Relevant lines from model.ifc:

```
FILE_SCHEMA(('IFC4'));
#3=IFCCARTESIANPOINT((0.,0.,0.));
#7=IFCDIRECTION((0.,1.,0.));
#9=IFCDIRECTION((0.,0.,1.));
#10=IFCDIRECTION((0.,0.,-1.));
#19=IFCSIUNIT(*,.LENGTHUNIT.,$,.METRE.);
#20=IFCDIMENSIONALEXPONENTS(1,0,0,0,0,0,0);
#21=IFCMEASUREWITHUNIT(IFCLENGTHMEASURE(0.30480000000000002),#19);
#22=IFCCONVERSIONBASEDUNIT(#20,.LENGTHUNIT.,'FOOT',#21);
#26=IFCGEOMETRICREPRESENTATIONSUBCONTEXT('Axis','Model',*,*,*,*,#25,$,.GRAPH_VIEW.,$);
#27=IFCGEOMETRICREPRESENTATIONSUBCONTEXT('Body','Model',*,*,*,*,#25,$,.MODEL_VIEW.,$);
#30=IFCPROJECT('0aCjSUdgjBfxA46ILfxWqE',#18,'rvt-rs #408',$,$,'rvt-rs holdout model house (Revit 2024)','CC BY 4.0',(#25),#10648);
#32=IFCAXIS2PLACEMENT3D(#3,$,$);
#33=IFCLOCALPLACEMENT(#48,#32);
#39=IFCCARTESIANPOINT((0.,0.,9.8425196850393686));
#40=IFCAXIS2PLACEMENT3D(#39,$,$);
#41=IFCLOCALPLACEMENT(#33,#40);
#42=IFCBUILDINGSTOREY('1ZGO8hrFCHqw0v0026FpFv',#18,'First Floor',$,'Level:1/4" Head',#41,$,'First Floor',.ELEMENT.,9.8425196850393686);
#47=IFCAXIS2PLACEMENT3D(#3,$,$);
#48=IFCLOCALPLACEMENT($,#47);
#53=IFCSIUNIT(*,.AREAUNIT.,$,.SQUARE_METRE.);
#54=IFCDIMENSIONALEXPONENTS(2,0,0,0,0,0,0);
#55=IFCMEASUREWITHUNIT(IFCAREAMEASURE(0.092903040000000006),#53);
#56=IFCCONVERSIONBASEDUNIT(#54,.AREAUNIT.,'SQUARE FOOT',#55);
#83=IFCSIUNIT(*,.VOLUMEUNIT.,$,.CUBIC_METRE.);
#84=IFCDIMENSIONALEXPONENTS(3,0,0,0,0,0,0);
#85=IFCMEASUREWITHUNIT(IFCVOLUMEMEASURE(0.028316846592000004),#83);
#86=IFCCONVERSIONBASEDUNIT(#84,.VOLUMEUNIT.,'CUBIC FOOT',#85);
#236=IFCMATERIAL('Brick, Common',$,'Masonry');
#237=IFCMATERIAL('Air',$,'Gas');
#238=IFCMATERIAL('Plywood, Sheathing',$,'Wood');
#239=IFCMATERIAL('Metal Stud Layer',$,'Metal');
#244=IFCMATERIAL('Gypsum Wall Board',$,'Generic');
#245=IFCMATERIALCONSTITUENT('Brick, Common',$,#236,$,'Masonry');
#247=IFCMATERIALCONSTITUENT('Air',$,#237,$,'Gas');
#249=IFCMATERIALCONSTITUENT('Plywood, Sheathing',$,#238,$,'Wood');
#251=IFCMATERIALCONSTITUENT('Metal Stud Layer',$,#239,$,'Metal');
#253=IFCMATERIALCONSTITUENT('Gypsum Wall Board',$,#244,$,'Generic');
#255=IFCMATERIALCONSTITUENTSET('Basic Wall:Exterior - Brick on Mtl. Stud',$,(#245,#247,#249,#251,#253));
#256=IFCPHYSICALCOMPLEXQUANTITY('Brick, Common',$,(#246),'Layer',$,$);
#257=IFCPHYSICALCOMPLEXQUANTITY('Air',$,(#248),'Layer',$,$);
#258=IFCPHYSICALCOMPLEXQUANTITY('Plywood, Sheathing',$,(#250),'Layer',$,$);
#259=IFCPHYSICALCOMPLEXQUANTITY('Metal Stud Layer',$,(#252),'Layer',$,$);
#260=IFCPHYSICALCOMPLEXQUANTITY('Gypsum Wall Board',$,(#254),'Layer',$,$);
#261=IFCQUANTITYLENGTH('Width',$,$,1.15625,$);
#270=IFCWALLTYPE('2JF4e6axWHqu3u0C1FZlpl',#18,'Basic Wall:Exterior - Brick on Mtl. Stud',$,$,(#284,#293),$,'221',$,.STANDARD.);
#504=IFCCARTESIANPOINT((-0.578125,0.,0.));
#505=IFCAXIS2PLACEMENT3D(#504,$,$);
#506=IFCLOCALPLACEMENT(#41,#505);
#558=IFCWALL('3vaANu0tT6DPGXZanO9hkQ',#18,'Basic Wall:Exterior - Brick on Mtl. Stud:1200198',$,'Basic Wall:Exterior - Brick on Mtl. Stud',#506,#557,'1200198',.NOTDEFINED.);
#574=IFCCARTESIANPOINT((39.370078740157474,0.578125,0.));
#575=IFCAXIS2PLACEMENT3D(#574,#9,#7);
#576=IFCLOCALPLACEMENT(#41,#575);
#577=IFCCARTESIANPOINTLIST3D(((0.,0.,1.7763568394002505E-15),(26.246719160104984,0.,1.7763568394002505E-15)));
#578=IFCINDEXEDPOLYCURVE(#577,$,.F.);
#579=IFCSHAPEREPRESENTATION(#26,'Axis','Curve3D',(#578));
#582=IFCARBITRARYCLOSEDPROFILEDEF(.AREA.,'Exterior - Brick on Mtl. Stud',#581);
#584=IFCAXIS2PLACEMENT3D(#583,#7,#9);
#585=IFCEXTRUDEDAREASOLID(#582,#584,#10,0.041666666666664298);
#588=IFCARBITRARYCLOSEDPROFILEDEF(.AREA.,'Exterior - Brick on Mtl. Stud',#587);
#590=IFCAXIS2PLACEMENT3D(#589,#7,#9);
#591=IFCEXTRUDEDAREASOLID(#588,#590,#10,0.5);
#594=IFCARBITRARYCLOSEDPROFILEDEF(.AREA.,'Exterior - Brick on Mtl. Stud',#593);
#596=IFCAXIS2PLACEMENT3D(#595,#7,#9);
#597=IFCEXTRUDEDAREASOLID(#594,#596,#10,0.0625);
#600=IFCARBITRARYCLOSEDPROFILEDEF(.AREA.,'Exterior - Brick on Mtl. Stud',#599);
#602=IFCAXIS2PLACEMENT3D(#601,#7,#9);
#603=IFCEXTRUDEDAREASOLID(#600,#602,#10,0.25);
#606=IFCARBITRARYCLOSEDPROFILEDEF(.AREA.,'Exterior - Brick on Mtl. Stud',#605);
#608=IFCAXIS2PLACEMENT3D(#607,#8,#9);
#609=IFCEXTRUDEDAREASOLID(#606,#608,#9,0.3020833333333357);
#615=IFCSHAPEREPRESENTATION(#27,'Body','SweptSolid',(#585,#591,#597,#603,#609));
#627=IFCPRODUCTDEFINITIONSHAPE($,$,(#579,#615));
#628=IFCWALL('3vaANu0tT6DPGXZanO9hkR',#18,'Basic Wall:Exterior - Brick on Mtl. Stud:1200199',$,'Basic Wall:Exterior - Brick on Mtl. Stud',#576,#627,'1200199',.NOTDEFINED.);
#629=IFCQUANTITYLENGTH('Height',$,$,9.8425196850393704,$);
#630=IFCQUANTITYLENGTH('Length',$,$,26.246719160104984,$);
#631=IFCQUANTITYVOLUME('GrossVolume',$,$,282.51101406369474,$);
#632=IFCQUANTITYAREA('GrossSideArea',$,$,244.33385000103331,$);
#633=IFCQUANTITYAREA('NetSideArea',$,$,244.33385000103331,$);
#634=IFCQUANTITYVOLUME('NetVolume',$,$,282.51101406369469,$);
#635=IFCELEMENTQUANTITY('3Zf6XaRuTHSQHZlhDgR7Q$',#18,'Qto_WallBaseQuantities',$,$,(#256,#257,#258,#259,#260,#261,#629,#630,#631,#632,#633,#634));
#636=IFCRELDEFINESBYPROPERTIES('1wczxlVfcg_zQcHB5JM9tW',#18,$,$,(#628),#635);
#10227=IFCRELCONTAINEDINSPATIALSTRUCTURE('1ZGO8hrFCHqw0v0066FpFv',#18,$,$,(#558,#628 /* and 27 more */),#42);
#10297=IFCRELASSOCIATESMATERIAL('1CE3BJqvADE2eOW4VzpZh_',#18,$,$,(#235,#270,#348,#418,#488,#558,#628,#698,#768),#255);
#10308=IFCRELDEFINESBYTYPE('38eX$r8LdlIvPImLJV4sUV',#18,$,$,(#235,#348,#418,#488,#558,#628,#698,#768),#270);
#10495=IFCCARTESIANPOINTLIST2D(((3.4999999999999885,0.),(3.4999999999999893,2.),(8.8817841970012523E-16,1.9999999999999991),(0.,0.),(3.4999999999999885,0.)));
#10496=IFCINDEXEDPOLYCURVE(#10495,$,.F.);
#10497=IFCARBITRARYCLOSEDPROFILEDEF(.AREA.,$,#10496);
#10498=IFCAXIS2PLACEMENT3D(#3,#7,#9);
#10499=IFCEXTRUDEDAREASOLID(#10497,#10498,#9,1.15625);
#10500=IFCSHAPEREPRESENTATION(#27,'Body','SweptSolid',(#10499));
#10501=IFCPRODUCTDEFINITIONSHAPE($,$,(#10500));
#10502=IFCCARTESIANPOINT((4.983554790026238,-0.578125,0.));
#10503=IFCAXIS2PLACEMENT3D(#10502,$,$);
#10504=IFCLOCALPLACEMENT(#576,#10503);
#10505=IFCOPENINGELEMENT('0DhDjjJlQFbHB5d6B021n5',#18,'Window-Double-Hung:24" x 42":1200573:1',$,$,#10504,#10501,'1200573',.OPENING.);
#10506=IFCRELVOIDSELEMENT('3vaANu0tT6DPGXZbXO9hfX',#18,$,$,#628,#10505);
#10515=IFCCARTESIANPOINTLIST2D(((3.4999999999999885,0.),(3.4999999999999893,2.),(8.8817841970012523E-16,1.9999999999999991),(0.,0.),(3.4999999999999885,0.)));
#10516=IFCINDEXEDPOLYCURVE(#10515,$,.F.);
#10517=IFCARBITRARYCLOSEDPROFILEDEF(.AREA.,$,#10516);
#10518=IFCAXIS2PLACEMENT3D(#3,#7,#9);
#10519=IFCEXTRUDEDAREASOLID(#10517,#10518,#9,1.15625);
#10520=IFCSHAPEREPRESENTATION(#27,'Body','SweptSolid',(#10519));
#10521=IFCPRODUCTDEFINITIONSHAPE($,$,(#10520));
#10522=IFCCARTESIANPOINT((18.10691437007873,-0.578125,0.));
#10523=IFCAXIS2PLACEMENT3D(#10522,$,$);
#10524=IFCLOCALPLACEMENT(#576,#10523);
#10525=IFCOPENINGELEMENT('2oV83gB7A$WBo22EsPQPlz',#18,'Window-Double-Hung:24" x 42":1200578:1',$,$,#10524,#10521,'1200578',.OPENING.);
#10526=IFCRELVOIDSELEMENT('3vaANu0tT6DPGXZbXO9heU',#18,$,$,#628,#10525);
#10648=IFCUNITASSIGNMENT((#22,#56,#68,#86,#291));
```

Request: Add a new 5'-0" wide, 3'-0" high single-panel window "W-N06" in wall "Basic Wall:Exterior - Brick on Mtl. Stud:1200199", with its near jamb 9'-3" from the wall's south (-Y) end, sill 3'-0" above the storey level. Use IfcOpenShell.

```python
import numpy as np
import ifcopenshell
import ifcopenshell.api.feature
import ifcopenshell.api.geometry
import ifcopenshell.api.pset
import ifcopenshell.api.root
import ifcopenshell.api.spatial
import ifcopenshell.geom
import ifcopenshell.util.element
import ifcopenshell.util.placement
import ifcopenshell.util.representation
import ifcopenshell.util.shape
import ifcopenshell.util.unit

model = ifcopenshell.open("model.ifc")
unit_scale = ifcopenshell.util.unit.calculate_unit_scale(model)
area_scale = ifcopenshell.util.unit.calculate_unit_scale(model, "AREAUNIT")
volume_scale = ifcopenshell.util.unit.calculate_unit_scale(model, "VOLUMEUNIT")
settings = ifcopenshell.geom.settings()


def volume(element):
    """Net volume in cubic metres, openings subtracted."""
    shape = ifcopenshell.geom.create_shape(settings, element)
    return ifcopenshell.util.shape.get_volume(shape.geometry)


wall = model.by_guid("3vaANu0tT6DPGXZanO9hkR")
storey = ifcopenshell.util.element.get_container(wall, ifc_class="IfcBuildingStorey")
context = ifcopenshell.util.representation.get_context(model, "Model", "Body", "MODEL_VIEW")
before = volume(wall)

width, height, from_end, sill = 1.524, 0.9144, 2.8194, 0.9144  # metres

# The wall runs along its own X axis, and the end named is its -X end.
wall_shape = ifcopenshell.geom.create_shape(settings, wall)
x, y, z = ifcopenshell.util.shape.get_vertices(wall_shape.geometry).T
start = x.min() + from_end
face, thickness = float(y.min()), float(y.max() - y.min())
wall_matrix = ifcopenshell.util.placement.get_local_placement(wall.ObjectPlacement)
level = ifcopenshell.util.placement.get_local_placement(storey.ObjectPlacement)[2, 3]


def in_wall(x, y):
    """Placement at x, y metres in the wall's axes, at sill height."""
    matrix = wall_matrix.copy()
    matrix[:, 3] = wall_matrix @ np.array([x / unit_scale, y / unit_scale, 0.0, 1.0])
    matrix[2, 3] = level + sill / unit_scale
    return matrix


# Opening: a box that overshoots both wall faces by 50 mm.
opening = ifcopenshell.api.root.create_entity(model, ifc_class="IfcOpeningElement", predefined_type="OPENING")
box = ifcopenshell.api.geometry.add_wall_representation(
    model, context=context, length=width, height=height, thickness=thickness + 0.1
)
ifcopenshell.api.geometry.assign_representation(model, product=opening, representation=box)
ifcopenshell.api.geometry.edit_object_placement(model, product=opening, matrix=in_wall(start, face - 0.05), is_si=False)
ifcopenshell.api.feature.add_feature(model, feature=opening, element=wall)

window = ifcopenshell.api.root.create_entity(model, ifc_class="IfcWindow", name="W-N06", predefined_type="WINDOW")
window.OverallWidth, window.OverallHeight = width / unit_scale, height / unit_scale
window.PartitioningType = "SINGLE_PANEL"
body = ifcopenshell.api.geometry.add_window_representation(
    model,
    context=context,
    overall_width=window.OverallWidth,
    overall_height=window.OverallHeight,
    partition_type="SINGLE_PANEL",
)
ifcopenshell.api.geometry.assign_representation(model, product=window, representation=body)
ifcopenshell.api.spatial.assign_container(model, products=[window], relating_structure=storey)
ifcopenshell.api.feature.add_filling(model, opening=opening, element=window)

# Centre the window in the wall's thickness.
ifcopenshell.api.geometry.edit_object_placement(model, product=window, matrix=in_wall(start, face), is_si=False)
window_shape = ifcopenshell.geom.create_shape(settings, window)
depth = ifcopenshell.util.shape.get_vertices(window_shape.geometry)[:, 1]
offset = face + thickness / 2 - (depth.min() + depth.max()) / 2
ifcopenshell.api.geometry.edit_object_placement(model, product=window, matrix=in_wall(start, offset), is_si=False)

after = volume(wall)

# Update the wall's stored quantities.
qto = model.by_id(ifcopenshell.util.element.get_pset(wall, "Qto_WallBaseQuantities", should_inherit=False)["id"])
ifcopenshell.api.pset.edit_qto(model, qto=qto, properties={
    "NetSideArea": after / thickness / area_scale,
    "NetVolume": after / volume_scale,
})

print(f"wall volume {before:.3f} -> {after:.3f} m3")

model.write("model_updated.ifc")
```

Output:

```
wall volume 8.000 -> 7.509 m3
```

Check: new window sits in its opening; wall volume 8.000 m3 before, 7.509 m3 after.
